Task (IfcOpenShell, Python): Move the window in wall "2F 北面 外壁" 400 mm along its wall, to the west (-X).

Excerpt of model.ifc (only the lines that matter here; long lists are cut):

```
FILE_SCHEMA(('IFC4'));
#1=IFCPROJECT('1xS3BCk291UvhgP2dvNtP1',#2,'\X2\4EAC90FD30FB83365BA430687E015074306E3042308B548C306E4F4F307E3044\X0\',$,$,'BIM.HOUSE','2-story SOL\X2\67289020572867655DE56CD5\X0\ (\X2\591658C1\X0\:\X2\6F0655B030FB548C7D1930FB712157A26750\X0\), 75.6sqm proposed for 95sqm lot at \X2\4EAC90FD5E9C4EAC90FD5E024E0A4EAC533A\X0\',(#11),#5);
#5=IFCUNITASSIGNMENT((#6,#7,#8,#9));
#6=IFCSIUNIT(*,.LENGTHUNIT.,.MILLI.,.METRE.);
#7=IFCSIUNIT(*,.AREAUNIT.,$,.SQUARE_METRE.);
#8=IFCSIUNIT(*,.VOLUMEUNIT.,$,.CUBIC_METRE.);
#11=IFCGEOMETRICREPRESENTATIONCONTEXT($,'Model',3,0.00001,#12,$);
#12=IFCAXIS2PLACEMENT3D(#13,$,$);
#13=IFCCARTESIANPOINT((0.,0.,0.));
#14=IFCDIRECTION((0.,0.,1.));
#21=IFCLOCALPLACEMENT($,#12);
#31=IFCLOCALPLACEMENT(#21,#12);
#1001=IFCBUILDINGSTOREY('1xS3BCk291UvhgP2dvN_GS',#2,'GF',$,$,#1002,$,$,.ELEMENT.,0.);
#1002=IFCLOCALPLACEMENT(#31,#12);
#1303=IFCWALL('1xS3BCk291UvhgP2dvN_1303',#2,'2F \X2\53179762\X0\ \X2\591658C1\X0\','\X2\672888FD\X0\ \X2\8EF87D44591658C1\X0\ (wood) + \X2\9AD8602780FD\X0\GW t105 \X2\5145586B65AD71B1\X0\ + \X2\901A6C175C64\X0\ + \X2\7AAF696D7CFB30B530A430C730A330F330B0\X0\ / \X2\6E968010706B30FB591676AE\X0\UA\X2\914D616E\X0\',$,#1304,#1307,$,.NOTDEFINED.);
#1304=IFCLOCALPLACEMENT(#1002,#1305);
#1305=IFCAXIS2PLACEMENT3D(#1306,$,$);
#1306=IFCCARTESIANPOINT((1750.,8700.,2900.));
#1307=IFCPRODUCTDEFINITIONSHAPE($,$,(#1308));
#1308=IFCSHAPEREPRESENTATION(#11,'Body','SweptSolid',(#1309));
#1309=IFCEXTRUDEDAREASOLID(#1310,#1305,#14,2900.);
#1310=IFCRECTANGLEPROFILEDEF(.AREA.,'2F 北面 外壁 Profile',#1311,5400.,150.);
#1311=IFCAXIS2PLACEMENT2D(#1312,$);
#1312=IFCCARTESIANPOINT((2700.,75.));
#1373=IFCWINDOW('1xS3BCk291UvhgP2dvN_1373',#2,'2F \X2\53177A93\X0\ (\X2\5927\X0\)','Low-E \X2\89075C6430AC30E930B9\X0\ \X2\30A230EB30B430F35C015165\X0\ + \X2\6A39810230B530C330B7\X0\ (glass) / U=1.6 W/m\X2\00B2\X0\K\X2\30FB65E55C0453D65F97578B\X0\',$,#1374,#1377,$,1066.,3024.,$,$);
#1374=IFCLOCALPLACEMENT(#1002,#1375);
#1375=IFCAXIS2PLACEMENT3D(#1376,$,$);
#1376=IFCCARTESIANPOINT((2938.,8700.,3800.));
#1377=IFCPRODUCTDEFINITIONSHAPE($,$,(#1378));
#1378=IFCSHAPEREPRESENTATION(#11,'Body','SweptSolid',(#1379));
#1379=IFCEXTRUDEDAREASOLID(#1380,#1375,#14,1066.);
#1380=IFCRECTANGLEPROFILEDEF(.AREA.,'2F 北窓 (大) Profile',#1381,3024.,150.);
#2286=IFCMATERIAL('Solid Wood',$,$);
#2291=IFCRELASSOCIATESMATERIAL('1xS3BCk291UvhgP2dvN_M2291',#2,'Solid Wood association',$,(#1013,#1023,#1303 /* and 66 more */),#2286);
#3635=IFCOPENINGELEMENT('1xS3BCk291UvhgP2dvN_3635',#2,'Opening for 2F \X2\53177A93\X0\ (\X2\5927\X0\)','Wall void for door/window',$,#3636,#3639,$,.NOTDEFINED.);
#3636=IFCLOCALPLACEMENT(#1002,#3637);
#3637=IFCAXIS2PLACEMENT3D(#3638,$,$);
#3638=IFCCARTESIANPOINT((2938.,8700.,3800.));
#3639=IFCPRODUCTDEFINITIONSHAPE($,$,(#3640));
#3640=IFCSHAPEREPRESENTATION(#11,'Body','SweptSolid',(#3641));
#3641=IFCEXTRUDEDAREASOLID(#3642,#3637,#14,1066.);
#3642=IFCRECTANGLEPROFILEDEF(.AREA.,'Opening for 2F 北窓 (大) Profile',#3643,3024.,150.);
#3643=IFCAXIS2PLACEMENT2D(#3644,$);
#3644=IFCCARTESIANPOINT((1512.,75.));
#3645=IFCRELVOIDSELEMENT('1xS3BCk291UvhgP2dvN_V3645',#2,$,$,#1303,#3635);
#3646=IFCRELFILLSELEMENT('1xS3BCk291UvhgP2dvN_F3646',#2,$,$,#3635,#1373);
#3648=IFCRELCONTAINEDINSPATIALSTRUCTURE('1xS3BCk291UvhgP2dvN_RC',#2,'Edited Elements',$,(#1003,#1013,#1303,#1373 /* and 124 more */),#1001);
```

```python
import ifcopenshell
import ifcopenshell.api.geometry
import ifcopenshell.util.placement

model = ifcopenshell.open("model.ifc")

window = model.by_guid("1xS3BCk291UvhgP2dvN_1373")
opening = window.FillsVoids[0].RelatingOpeningElement
wall = opening.VoidsElements[0].RelatingBuildingElement

wall_matrix = ifcopenshell.util.placement.get_local_placement(wall.ObjectPlacement)
shift = wall_matrix[:3, 0] * -400.0
before = ifcopenshell.util.placement.get_local_placement(window.ObjectPlacement)[:3, 3].copy()

# The window is not placed relative to its opening, so move both.
for product in (opening, window):
    matrix = ifcopenshell.util.placement.get_local_placement(product.ObjectPlacement)
    matrix[:3, 3] += shift
    ifcopenshell.api.geometry.edit_object_placement(model, product=product, matrix=matrix, is_si=False)

after = ifcopenshell.util.placement.get_local_placement(window.ObjectPlacement)[:3, 3]
print("window moved by", (after - before).round(3) + 0.0)

model.write("model_updated.ifc")
```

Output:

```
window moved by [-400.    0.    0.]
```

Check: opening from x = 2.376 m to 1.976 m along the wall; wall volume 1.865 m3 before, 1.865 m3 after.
